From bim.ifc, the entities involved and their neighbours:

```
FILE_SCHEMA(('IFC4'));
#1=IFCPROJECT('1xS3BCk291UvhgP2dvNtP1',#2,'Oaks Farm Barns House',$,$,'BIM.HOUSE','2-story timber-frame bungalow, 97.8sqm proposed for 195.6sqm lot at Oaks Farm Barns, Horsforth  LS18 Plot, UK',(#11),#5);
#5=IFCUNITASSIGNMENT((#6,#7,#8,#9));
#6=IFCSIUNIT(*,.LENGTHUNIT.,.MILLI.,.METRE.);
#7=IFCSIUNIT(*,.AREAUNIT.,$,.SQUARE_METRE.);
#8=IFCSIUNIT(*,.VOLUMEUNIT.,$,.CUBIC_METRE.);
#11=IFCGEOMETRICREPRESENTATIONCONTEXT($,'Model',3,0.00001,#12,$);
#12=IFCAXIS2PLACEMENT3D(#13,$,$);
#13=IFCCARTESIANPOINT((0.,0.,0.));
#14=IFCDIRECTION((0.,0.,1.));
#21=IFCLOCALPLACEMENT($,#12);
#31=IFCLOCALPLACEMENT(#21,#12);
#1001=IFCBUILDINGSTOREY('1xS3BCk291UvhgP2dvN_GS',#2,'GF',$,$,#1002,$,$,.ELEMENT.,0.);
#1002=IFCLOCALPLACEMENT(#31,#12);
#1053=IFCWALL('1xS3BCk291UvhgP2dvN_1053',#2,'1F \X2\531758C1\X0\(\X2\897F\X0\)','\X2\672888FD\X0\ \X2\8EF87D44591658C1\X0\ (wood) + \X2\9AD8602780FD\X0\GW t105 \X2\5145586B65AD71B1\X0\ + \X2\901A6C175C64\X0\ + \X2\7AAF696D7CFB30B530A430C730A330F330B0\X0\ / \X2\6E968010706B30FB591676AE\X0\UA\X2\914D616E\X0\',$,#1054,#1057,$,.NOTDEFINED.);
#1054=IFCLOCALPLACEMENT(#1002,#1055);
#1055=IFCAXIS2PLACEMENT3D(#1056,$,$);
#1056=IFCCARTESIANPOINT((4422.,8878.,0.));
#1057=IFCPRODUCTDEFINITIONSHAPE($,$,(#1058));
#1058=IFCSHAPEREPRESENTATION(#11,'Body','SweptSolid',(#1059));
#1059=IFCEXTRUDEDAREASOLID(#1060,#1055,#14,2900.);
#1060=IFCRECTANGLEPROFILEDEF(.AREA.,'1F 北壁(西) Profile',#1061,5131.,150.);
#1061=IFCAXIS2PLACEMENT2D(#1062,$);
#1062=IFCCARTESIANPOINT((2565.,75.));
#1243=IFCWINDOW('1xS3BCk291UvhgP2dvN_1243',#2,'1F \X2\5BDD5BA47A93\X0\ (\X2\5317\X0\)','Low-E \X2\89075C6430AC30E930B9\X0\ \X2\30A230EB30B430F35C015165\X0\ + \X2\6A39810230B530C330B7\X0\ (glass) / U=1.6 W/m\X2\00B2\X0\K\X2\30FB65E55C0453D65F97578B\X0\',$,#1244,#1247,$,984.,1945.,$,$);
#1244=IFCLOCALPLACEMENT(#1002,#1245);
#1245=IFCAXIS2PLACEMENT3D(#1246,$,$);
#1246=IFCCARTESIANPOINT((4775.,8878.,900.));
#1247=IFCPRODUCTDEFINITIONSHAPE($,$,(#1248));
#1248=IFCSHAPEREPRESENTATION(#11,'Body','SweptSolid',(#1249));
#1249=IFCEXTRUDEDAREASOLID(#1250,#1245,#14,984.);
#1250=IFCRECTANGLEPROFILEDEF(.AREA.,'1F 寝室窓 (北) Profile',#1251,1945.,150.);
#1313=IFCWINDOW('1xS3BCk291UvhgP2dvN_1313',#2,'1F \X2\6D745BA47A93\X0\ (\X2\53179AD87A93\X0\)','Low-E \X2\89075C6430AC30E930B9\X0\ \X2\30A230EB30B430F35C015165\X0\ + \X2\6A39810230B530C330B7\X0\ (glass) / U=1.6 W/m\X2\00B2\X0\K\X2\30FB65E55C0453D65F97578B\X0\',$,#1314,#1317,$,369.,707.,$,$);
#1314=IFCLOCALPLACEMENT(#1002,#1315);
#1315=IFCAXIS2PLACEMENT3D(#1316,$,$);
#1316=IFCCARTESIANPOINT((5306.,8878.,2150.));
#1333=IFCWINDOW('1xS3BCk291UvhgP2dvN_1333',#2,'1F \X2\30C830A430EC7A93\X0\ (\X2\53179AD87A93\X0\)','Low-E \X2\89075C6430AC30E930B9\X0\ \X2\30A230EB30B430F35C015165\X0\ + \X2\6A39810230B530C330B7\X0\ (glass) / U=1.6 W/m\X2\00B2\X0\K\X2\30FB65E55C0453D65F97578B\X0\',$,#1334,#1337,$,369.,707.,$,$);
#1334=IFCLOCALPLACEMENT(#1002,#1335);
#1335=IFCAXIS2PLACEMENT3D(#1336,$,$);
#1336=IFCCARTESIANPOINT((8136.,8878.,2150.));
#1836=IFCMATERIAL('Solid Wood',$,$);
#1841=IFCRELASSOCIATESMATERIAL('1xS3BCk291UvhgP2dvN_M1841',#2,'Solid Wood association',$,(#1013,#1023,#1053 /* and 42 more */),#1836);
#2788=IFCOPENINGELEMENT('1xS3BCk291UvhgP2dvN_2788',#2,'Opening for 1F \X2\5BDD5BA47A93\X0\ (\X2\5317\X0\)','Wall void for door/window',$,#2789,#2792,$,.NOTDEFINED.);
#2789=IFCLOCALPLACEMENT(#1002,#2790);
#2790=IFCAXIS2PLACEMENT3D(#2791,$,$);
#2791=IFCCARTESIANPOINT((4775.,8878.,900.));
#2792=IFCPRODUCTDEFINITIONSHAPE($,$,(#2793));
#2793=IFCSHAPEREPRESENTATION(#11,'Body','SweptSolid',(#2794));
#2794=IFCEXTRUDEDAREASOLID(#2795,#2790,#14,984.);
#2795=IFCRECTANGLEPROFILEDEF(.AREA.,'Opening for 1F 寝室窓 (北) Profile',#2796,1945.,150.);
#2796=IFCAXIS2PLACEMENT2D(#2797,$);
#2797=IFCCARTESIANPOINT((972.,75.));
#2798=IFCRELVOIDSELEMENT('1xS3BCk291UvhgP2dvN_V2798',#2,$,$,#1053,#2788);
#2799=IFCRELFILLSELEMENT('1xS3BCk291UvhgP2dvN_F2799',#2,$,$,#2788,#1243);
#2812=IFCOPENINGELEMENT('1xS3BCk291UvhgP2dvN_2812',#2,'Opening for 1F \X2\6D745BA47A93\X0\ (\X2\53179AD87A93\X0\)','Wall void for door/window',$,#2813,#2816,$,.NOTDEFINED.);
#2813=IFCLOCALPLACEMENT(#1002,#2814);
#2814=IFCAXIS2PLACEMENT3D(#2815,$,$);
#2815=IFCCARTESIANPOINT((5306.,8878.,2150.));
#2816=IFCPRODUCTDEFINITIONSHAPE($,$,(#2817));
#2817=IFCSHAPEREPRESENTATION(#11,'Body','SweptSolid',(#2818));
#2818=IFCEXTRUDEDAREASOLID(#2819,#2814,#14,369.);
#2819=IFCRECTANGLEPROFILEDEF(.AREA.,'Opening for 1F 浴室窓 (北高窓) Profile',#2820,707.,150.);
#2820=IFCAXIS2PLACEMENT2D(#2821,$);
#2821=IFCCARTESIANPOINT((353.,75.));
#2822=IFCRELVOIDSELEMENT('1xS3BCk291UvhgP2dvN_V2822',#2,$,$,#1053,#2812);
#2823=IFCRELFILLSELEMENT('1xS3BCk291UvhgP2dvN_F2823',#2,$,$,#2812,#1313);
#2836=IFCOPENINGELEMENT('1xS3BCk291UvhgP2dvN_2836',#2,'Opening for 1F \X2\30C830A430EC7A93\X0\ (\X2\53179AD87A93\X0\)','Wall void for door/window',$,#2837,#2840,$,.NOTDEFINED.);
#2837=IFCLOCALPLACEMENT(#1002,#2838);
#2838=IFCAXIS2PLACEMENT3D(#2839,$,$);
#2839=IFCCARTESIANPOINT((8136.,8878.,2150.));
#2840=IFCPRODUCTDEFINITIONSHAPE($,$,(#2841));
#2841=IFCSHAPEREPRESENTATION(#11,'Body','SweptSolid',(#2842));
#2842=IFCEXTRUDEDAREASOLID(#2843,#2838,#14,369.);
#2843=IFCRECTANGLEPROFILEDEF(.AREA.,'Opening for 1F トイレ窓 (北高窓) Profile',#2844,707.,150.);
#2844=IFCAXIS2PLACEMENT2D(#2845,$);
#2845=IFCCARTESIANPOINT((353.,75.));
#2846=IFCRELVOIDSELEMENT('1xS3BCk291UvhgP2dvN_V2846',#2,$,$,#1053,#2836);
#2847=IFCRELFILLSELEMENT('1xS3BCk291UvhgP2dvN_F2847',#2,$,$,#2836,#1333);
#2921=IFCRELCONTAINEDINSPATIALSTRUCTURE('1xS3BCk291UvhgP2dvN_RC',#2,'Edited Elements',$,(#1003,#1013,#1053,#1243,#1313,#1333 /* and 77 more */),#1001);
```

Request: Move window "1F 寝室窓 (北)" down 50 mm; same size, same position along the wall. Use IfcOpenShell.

```python
import numpy as np
import ifcopenshell
import ifcopenshell.api.geometry
import ifcopenshell.util.placement
import ifcopenshell.util.unit

model = ifcopenshell.open("bim.ifc")
unit_scale = ifcopenshell.util.unit.calculate_unit_scale(model)

window = model.by_guid("1xS3BCk291UvhgP2dvN_1243")
opening = window.FillsVoids[0].RelatingOpeningElement
dz = -50.0

shift = np.array([0.0, 0.0, dz])
# The window is not placed relative to its opening, so move both.
for product in (opening, window):
    matrix = ifcopenshell.util.placement.get_local_placement(product.ObjectPlacement)
    matrix[:3, 3] += shift
    ifcopenshell.api.geometry.edit_object_placement(model, product=product, matrix=matrix, is_si=False)

print(f"moved by {dz * unit_scale:+.3f} m")

model.write("bim_updated.ifc")
```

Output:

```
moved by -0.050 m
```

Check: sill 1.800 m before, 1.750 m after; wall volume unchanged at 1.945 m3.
